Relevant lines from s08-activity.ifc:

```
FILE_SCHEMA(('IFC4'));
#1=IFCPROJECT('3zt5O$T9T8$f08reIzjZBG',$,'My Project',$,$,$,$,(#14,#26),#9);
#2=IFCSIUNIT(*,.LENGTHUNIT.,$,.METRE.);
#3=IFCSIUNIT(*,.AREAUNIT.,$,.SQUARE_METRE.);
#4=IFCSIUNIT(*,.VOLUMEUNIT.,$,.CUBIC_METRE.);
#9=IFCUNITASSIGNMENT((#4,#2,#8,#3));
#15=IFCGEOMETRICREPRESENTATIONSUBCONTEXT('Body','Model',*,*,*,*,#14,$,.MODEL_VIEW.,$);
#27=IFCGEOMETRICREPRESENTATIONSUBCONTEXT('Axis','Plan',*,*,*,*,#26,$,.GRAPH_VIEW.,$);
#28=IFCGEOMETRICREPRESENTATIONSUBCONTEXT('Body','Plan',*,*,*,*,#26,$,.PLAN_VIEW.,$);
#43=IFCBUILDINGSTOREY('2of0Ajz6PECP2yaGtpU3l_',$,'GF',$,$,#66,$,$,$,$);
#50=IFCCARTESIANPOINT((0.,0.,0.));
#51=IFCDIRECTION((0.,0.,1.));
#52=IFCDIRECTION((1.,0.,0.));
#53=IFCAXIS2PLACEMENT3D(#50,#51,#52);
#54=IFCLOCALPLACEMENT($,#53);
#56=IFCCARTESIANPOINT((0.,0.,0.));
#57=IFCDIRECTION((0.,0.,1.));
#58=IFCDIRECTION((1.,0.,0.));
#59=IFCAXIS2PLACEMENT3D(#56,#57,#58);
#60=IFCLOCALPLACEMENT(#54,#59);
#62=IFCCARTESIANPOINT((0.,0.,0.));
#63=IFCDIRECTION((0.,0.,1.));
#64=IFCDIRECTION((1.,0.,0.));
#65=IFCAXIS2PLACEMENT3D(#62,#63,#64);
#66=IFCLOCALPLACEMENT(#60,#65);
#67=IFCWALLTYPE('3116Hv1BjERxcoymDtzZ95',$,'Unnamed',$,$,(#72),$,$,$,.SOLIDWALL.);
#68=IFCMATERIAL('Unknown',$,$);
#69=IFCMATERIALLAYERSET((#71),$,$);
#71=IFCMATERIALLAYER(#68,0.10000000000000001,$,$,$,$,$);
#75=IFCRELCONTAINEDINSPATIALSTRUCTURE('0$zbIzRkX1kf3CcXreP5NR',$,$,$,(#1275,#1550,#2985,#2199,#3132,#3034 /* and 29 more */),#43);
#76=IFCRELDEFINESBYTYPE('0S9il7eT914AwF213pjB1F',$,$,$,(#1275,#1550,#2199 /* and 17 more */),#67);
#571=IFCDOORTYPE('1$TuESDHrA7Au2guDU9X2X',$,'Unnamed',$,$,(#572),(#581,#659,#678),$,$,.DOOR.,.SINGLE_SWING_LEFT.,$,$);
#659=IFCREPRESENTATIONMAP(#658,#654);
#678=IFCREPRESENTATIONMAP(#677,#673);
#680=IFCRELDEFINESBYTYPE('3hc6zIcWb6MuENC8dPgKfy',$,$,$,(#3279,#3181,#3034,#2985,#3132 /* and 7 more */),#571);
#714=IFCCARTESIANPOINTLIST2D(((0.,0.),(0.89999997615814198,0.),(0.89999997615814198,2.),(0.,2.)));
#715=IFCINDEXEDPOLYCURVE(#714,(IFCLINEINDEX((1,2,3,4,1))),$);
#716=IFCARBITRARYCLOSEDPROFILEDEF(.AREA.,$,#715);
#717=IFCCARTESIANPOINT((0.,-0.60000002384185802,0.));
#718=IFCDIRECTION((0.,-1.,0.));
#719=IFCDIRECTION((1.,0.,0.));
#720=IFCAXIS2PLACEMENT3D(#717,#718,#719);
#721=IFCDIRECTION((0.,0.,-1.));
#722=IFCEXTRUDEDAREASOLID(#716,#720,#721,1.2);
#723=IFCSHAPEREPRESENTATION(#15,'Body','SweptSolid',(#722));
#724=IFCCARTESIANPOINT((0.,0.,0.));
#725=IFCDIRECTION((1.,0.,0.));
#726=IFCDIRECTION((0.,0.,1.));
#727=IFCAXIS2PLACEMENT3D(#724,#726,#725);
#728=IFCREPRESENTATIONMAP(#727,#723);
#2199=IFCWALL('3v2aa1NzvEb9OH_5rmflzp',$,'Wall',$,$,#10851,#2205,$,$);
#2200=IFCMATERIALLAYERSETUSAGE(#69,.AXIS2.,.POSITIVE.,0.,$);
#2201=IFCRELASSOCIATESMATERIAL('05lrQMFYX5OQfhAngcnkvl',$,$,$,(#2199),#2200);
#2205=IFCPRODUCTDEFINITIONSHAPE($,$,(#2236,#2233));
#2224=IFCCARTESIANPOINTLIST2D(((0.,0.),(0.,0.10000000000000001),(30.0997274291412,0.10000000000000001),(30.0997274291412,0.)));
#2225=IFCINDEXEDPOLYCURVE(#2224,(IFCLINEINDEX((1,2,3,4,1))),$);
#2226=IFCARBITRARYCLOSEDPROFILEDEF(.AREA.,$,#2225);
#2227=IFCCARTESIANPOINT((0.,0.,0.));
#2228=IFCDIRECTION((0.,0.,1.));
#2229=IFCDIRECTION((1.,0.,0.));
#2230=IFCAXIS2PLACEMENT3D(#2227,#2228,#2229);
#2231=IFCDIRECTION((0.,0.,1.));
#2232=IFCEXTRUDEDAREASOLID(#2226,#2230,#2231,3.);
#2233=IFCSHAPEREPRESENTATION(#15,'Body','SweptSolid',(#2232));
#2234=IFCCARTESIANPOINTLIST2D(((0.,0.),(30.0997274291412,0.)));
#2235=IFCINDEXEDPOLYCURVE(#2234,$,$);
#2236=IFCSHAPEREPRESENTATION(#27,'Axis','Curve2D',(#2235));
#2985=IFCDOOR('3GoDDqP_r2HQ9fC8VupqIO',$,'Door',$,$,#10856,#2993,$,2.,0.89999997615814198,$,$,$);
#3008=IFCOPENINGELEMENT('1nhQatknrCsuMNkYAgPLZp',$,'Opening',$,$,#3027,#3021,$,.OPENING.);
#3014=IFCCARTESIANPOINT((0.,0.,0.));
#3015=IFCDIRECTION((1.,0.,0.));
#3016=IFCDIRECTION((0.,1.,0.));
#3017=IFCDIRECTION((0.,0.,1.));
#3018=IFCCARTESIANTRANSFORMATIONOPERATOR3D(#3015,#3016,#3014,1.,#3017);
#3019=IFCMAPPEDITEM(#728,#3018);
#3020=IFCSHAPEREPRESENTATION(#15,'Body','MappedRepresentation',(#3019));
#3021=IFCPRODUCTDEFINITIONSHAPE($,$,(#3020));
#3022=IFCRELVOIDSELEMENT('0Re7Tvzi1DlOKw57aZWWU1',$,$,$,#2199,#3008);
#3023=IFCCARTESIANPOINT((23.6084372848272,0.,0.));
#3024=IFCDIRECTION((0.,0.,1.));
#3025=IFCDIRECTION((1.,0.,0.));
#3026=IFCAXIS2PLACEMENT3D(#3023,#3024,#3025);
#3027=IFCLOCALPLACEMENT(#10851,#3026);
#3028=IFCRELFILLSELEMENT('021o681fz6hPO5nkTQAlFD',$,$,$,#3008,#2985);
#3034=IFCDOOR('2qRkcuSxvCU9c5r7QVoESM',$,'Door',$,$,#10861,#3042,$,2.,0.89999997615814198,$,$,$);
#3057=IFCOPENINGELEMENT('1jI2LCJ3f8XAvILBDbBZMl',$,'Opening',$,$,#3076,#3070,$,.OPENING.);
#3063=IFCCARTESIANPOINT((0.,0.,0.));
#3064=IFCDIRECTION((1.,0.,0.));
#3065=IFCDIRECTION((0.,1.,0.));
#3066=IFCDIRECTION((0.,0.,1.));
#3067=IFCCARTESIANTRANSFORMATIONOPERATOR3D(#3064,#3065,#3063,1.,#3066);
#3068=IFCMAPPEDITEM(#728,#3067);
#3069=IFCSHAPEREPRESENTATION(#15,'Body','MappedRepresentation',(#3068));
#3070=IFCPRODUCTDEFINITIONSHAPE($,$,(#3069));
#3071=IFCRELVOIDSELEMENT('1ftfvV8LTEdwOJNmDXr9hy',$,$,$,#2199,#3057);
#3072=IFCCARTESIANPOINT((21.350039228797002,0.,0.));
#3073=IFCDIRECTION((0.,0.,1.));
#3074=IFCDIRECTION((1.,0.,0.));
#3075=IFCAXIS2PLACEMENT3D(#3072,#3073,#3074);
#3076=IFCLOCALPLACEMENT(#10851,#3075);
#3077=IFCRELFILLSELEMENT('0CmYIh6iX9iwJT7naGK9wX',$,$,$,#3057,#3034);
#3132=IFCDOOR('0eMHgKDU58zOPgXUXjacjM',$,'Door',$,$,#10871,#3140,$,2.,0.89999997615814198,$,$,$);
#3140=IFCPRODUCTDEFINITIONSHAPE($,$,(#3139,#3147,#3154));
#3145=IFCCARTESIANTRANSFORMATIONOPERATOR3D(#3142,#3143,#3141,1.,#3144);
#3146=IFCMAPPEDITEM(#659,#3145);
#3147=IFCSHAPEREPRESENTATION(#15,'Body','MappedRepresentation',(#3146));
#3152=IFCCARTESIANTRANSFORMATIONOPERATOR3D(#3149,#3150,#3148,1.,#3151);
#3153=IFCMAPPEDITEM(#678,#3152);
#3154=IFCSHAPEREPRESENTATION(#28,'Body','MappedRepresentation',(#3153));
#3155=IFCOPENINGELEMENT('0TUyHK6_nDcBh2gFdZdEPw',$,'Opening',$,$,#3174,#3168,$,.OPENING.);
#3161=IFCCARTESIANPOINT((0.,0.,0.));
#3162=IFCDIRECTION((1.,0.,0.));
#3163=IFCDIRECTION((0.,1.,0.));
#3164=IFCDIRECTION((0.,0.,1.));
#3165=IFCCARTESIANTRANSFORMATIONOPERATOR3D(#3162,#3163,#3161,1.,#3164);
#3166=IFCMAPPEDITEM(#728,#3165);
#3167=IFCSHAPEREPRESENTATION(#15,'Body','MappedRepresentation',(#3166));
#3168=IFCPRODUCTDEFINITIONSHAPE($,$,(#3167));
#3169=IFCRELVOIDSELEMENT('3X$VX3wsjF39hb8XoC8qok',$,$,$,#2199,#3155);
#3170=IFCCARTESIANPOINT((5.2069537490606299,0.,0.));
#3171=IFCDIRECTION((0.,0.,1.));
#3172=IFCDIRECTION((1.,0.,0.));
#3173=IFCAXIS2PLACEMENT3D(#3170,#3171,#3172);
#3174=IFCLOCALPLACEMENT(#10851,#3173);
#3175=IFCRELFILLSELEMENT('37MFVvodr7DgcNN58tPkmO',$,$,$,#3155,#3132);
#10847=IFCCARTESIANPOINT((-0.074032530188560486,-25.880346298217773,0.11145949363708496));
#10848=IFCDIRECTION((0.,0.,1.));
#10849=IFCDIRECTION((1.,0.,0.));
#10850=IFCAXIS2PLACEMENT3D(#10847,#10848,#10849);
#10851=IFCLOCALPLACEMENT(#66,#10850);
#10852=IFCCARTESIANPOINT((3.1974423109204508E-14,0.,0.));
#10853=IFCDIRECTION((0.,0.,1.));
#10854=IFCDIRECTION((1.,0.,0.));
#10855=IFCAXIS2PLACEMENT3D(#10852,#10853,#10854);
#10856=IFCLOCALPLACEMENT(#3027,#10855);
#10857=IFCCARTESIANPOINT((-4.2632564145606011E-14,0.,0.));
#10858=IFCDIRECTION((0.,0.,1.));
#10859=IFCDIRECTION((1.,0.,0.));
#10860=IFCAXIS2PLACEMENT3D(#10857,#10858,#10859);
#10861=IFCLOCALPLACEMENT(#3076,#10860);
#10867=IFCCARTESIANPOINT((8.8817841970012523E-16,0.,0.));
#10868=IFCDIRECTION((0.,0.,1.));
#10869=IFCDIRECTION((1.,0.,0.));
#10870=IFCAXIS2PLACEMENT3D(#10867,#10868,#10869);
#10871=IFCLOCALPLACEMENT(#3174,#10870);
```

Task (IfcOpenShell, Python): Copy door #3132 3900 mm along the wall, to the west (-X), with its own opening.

```python
import ifcopenshell
import ifcopenshell.api.feature
import ifcopenshell.api.geometry
import ifcopenshell.api.root
import ifcopenshell.geom
import ifcopenshell.util.element
import ifcopenshell.util.placement
import ifcopenshell.util.shape

model = ifcopenshell.open("s08-activity.ifc")
settings = ifcopenshell.geom.settings()


def volume(element):
    """Net volume in cubic metres, openings subtracted."""
    shape = ifcopenshell.geom.create_shape(settings, element)
    return ifcopenshell.util.shape.get_volume(shape.geometry)


door = model.by_id(3132)
opening = door.FillsVoids[0].RelatingOpeningElement
wall = opening.VoidsElements[0].RelatingBuildingElement
before = volume(wall)
shift = ifcopenshell.util.placement.get_local_placement(wall.ObjectPlacement)[:3, 0] * -3.9

# copy_class copies the void relationship, type, container and properties, but no geometry.
new_opening = ifcopenshell.api.root.copy_class(model, product=opening)
new_opening.Representation = ifcopenshell.util.element.copy_deep(
    model, opening.Representation, exclude=["IfcGeometricRepresentationContext", "IfcRepresentationMap"]
)
new_door = ifcopenshell.api.root.copy_class(model, product=door)
new_door.Representation = ifcopenshell.util.element.copy_deep(
    model, door.Representation, exclude=["IfcGeometricRepresentationContext", "IfcRepresentationMap"]
)
ifcopenshell.api.feature.add_filling(model, opening=new_opening, element=new_door)

for old, new in ((opening, new_opening), (door, new_door)):
    matrix = ifcopenshell.util.placement.get_local_placement(old.ObjectPlacement)
    matrix[:3, 3] += shift
    ifcopenshell.api.geometry.edit_object_placement(model, product=new, matrix=matrix, is_si=False)

after = volume(wall)

print(f"wall volume {before:.3f} -> {after:.3f} m3")

model.write("s08-activity_updated.ifc")
```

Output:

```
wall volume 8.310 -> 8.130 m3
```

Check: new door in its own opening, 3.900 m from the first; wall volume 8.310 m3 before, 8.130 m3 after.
